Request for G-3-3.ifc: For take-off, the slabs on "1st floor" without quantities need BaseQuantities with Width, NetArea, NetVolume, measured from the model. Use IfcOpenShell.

First a look at what the model holds.

```python
import ifcopenshell
import ifcopenshell.util.element
import ifcopenshell.util.unit

model = ifcopenshell.open("G-3-3.ifc")
print(model.schema)
for unit_type in ("LENGTHUNIT", "AREAUNIT", "VOLUMEUNIT"):
    print(unit_type, ifcopenshell.util.unit.calculate_unit_scale(model, unit_type))
storey = next(s for s in model.by_type("IfcBuildingStorey") if s.Name == "1st floor")
slabs = [e for e in ifcopenshell.util.element.get_decomposition(storey) if e.is_a("IfcSlab")]
for e in sorted(slabs, key=lambda e: e.id()):
    print(e.id(), e.is_a(), e.Name, list(ifcopenshell.util.element.get_psets(e, qtos_only=True)), sep=" | ")
```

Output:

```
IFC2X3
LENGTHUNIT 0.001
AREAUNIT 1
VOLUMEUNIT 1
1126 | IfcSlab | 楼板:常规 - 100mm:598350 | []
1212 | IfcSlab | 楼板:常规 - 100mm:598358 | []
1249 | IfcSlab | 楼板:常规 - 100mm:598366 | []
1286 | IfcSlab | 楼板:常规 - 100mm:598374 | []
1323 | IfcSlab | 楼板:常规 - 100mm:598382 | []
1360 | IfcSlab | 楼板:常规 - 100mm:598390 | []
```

```python
import ifcopenshell
import ifcopenshell.api.pset
import ifcopenshell.geom
import ifcopenshell.util.element
import ifcopenshell.util.shape
import ifcopenshell.util.unit

model = ifcopenshell.open("G-3-3.ifc")
unit_scale = ifcopenshell.util.unit.calculate_unit_scale(model)
area_scale = ifcopenshell.util.unit.calculate_unit_scale(model, "AREAUNIT")
volume_scale = ifcopenshell.util.unit.calculate_unit_scale(model, "VOLUMEUNIT")
settings = ifcopenshell.geom.settings()

storey = next(s for s in model.by_type("IfcBuildingStorey") if s.Name == "1st floor")
slabs = [e for e in ifcopenshell.util.element.get_decomposition(storey) if e.is_a("IfcSlab")]

for e in sorted(slabs, key=lambda e: e.id()):
    if ifcopenshell.util.element.get_psets(e, qtos_only=True, should_inherit=False):
        continue
    # Geometry comes back in metres, in the element's own axes.
    shape = ifcopenshell.geom.create_shape(settings, e)
    values = {
        "Width": ifcopenshell.util.shape.get_z(shape.geometry) / unit_scale,
        "NetArea": ifcopenshell.util.shape.get_footprint_area(shape.geometry) / area_scale,
        "NetVolume": ifcopenshell.util.shape.get_volume(shape.geometry) / volume_scale,
    }
    qto = ifcopenshell.api.pset.add_qto(model, product=e, name="BaseQuantities")
    ifcopenshell.api.pset.edit_qto(model, qto=qto, properties=values)
    print(e.id(), {k: round(v, 3) for k, v in values.items()})

model.write("G-3-3_rev.ifc")
```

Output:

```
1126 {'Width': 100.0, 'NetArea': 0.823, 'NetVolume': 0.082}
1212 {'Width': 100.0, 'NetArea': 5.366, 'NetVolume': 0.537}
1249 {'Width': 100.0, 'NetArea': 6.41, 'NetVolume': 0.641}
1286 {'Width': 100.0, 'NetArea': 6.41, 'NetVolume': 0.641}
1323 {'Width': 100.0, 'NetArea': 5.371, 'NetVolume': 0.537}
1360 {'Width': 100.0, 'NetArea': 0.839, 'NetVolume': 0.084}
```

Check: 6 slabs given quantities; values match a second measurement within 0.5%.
